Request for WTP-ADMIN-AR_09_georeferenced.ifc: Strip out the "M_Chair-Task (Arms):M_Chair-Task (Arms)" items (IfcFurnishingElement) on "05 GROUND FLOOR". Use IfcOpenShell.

First a look at what the model holds.

```python
import ifcopenshell
import ifcopenshell.util.element

model = ifcopenshell.open("WTP-ADMIN-AR_09_georeferenced.ifc")
print(model.schema)
storey = next(s for s in model.by_type("IfcBuildingStorey") if s.Name == "05 GROUND FLOOR")
furniture = [e for e in ifcopenshell.util.element.get_decomposition(storey) if e.is_a("IfcFurnishingElement")]
seen = {}
for e in furniture:
    element_type = ifcopenshell.util.element.get_type(e)
    name = element_type.Name if element_type not in (None, e) else None
    seen[name] = seen.get(name, 0) + 1
for name, count in sorted(seen.items(), key=str):
    print(count, "x", name)
```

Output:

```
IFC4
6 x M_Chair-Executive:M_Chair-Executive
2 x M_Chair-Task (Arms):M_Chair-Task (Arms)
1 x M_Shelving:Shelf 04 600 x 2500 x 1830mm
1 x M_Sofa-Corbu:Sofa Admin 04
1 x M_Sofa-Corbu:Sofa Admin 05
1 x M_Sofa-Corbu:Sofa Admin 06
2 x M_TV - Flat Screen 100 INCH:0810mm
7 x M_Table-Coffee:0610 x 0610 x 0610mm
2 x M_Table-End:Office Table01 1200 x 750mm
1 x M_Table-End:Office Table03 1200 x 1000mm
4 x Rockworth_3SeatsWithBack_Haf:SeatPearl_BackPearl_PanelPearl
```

```python
import ifcopenshell
import ifcopenshell.api.root
import ifcopenshell.util.element

model = ifcopenshell.open("WTP-ADMIN-AR_09_georeferenced.ifc")

storey = next(s for s in model.by_type("IfcBuildingStorey") if s.Name == "05 GROUND FLOOR")
furniture = [e for e in ifcopenshell.util.element.get_decomposition(storey) if e.is_a("IfcFurnishingElement")]
targets = [e for e in furniture if (t := ifcopenshell.util.element.get_type(e)) not in (None, e) and t.Name == "M_Chair-Task (Arms):M_Chair-Task (Arms)"]

for e in targets:
    ifcopenshell.api.root.remove_product(model, product=e)
print(len(targets), "removed")

model.write("WTP-ADMIN-AR_09_georeferenced_v2.ifc")
```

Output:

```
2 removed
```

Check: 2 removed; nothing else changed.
